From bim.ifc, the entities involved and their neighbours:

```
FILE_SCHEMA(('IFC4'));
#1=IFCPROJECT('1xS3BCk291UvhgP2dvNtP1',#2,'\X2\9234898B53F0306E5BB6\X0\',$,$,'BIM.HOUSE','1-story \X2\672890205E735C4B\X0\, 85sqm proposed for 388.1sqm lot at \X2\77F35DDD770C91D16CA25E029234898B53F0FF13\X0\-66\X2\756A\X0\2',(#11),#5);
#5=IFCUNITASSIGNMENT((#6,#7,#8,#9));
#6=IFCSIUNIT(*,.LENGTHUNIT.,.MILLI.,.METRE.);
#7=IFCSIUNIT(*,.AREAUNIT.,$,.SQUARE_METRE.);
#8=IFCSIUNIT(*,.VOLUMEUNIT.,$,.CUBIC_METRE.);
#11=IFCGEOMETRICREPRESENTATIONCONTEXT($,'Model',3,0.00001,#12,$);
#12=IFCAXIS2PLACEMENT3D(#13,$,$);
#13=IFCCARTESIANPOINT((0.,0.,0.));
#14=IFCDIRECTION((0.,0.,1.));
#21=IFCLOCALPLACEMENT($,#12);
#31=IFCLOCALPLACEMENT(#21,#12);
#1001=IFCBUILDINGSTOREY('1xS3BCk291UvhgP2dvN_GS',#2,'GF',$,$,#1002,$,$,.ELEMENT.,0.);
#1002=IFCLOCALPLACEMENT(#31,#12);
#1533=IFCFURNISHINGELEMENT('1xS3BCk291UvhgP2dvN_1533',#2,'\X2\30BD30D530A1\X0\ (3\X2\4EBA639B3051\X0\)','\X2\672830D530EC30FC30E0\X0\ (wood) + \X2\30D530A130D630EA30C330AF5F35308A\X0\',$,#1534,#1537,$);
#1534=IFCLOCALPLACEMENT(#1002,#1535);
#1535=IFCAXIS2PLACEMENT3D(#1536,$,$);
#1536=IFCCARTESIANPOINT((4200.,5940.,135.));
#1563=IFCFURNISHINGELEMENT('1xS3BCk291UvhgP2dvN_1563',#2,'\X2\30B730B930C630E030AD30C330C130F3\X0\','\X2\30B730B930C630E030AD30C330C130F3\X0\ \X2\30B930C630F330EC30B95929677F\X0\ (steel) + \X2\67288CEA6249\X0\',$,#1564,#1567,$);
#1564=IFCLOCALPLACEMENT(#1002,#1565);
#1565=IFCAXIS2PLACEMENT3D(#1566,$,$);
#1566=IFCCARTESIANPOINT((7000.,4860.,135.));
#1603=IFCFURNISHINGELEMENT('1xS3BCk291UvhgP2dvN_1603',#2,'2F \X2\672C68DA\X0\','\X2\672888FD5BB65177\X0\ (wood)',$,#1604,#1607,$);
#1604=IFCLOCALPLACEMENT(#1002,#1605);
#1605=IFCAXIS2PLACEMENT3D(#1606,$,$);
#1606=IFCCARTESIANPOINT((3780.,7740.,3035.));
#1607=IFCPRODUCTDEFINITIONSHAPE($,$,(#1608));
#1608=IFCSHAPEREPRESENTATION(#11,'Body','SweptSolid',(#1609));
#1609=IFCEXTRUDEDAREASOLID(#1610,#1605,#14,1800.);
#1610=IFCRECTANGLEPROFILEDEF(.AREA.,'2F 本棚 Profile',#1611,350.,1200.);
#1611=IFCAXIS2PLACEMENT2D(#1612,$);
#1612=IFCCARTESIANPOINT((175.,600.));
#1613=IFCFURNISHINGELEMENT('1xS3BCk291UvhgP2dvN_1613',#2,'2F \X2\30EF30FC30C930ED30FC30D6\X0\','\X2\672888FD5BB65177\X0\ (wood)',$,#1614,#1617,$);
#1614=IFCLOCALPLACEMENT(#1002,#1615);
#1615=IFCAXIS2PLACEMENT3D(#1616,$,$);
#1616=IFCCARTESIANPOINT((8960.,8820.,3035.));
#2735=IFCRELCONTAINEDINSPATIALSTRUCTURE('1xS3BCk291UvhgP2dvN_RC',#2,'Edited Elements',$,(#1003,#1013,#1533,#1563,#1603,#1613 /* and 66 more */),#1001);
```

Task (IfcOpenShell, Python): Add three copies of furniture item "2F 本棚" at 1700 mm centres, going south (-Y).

```python
import numpy as np
import ifcopenshell
import ifcopenshell.api.geometry
import ifcopenshell.api.root
import ifcopenshell.util.element
import ifcopenshell.util.placement
import ifcopenshell.util.unit

model = ifcopenshell.open("bim.ifc")
unit_scale = ifcopenshell.util.unit.calculate_unit_scale(model)


def reuse_history(source, copy):
    """copy_class also copies each property set's owner history, people and application; keep the originals."""
    for rel in copy.IsDefinedBy:
        if rel.is_a("IfcRelDefinesByProperties") and (history := rel.RelatingPropertyDefinition.OwnerHistory):
            rel.RelatingPropertyDefinition.OwnerHistory = source.OwnerHistory
            ifcopenshell.util.element.remove_deep2(model, history)


source = model.by_guid("1xS3BCk291UvhgP2dvN_1603")
base = ifcopenshell.util.placement.get_local_placement(source.ObjectPlacement)
step = np.array([0.0, -1.0, 0.0]) * 1.7 / unit_scale

for i in range(1, 4):
    copy = ifcopenshell.api.root.copy_class(model, product=source)
    copy.Representation = ifcopenshell.util.element.copy_deep(
        model, source.Representation, exclude=["IfcGeometricRepresentationContext", "IfcRepresentationMap"]
    )
    reuse_history(source, copy)
    matrix = base.copy()
    matrix[:3, 3] += i * step
    print("added at", matrix[:3, 3].round(3) + 0.0)
    ifcopenshell.api.geometry.edit_object_placement(model, product=copy, matrix=matrix, is_si=False)

model.write("bim_updated.ifc")
```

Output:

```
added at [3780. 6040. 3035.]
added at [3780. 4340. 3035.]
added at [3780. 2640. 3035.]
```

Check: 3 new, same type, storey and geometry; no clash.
